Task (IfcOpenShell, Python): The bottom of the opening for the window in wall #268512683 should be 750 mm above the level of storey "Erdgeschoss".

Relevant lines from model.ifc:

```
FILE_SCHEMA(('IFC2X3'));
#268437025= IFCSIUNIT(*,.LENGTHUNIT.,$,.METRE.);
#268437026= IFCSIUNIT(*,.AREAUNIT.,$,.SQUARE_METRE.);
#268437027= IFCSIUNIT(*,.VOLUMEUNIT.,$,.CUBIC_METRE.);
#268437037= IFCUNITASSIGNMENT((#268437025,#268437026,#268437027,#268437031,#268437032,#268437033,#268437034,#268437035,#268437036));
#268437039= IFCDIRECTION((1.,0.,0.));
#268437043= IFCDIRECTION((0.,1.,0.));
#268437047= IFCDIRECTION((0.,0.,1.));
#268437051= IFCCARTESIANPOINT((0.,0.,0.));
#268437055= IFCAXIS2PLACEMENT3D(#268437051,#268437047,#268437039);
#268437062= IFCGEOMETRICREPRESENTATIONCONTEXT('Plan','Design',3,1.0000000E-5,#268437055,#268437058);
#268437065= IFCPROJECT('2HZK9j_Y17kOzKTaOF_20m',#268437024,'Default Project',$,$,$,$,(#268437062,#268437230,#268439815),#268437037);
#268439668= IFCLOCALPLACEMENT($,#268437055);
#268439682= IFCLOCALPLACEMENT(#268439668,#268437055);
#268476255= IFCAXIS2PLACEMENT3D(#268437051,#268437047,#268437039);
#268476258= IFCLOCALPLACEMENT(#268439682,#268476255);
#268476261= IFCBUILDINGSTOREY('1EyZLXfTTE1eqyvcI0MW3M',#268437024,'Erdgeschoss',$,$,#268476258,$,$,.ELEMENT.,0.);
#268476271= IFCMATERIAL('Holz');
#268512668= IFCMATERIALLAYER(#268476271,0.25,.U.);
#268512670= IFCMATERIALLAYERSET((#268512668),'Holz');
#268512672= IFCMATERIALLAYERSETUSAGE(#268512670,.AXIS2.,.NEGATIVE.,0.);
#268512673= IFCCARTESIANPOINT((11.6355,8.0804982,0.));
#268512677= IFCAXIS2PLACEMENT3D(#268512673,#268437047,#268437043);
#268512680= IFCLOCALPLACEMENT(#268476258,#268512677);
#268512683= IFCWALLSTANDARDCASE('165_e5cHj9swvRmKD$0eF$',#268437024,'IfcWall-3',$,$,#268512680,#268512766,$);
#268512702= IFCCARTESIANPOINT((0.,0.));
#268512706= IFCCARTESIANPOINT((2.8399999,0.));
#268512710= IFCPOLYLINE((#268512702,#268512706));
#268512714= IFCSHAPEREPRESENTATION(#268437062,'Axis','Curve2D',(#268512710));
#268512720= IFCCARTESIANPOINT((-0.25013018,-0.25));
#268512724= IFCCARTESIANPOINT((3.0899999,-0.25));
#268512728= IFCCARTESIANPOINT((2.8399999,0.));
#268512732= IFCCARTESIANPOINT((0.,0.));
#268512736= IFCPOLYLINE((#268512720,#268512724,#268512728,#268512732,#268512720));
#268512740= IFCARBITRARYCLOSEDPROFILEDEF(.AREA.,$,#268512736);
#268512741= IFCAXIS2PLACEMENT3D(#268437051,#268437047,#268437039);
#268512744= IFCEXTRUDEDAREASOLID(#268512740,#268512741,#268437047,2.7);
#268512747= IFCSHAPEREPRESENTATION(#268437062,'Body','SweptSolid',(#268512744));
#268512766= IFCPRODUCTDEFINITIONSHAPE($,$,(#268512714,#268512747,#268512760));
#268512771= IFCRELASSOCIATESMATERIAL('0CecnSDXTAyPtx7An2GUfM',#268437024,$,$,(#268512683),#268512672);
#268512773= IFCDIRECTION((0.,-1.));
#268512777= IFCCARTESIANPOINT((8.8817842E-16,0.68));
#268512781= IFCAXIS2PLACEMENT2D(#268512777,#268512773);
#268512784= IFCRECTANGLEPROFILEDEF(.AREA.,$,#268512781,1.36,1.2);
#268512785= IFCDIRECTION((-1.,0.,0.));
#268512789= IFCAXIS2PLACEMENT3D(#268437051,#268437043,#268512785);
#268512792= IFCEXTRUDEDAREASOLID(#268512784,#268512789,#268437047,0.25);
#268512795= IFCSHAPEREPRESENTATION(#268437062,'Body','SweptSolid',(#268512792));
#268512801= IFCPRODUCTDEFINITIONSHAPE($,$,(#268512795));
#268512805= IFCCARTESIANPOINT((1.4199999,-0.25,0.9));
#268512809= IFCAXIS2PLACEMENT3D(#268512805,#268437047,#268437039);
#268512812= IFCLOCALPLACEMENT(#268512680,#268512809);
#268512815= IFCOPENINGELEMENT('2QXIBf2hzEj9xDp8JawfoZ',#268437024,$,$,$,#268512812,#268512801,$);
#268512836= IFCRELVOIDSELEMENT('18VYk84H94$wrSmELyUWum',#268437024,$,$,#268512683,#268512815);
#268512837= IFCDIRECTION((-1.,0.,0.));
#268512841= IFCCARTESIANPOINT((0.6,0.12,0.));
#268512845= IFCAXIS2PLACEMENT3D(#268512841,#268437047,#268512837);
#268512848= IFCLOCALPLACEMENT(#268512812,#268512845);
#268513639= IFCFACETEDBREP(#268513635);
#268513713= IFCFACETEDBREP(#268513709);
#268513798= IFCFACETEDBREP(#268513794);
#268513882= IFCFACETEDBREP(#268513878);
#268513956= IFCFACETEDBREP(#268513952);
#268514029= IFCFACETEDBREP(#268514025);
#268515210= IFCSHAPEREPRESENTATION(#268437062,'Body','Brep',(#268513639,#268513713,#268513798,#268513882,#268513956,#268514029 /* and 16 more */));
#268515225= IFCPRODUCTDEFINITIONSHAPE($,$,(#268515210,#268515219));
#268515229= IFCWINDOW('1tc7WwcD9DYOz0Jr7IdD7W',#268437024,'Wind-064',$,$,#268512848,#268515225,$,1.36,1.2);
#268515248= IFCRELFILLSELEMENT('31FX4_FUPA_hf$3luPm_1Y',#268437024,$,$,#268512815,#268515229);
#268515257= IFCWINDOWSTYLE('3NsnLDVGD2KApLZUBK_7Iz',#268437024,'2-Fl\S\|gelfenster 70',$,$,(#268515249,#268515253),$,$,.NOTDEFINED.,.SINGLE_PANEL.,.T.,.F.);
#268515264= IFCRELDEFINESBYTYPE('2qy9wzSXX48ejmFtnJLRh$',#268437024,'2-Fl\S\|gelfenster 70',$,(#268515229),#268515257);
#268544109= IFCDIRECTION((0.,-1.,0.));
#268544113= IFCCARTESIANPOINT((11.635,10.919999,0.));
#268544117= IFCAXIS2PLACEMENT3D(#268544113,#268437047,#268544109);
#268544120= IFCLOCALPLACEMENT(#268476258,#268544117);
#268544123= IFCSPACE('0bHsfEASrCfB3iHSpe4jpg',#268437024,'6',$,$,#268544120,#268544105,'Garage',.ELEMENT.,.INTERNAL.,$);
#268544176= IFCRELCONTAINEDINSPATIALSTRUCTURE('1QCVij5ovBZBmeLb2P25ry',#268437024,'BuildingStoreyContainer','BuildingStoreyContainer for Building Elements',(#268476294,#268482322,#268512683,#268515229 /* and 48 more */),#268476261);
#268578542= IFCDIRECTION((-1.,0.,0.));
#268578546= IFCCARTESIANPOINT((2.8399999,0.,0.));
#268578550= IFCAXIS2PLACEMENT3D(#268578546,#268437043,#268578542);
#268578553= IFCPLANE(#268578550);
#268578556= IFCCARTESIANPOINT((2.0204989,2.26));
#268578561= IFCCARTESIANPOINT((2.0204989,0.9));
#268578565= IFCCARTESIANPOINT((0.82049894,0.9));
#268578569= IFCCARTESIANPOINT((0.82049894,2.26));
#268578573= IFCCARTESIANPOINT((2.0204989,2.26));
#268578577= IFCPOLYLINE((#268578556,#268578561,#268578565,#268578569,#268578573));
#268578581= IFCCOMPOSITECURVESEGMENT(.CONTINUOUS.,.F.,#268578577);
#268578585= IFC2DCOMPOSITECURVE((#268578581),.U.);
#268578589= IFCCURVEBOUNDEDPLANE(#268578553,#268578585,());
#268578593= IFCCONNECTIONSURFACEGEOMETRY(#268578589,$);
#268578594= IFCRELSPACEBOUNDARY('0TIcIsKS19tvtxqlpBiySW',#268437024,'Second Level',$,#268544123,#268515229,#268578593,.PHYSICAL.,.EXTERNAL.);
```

```python
import numpy as np
import ifcopenshell
import ifcopenshell.api.geometry
import ifcopenshell.geom
import ifcopenshell.util.element
import ifcopenshell.util.placement
import ifcopenshell.util.shape
import ifcopenshell.util.unit

model = ifcopenshell.open("model.ifc")
unit_scale = ifcopenshell.util.unit.calculate_unit_scale(model)

window = model.by_guid("1tc7WwcD9DYOz0Jr7IdD7W")
opening = window.FillsVoids[0].RelatingOpeningElement
storey = ifcopenshell.util.element.get_container(window, ifc_class="IfcBuildingStorey")
level = ifcopenshell.util.placement.get_local_placement(storey.ObjectPlacement)[2, 3]

# The opening's origin need not be at the sill, so measure its lowest point.
shape = ifcopenshell.geom.create_shape(ifcopenshell.geom.settings(), opening)
bottom = ifcopenshell.util.shape.get_shape_bottom_elevation(shape, shape.geometry) / unit_scale
dz = level + 0.75 / unit_scale - bottom

shift = np.array([0.0, 0.0, dz])
# The window is placed relative to its opening, so it follows when the opening moves.
matrix = ifcopenshell.util.placement.get_local_placement(opening.ObjectPlacement)
matrix[:3, 3] += shift
ifcopenshell.api.geometry.edit_object_placement(
    model, product=opening, matrix=matrix, is_si=False, should_transform_children=True
)

# Space boundary surfaces are stored in each space's coordinates; move them too.
for rel in window.ProvidesBoundaries:
    if not rel.ConnectionGeometry:
        continue
    surface = rel.ConnectionGeometry.SurfaceOnRelatingElement.BasisSurface
    space_matrix = ifcopenshell.util.placement.get_local_placement(rel.RelatingSpace.ObjectPlacement)
    point = np.array(surface.Position.Location.Coordinates) + space_matrix[:3, :3].T @ shift
    surface.Position = model.createIfcAxis2Placement3D(
        model.createIfcCartesianPoint(point.tolist()), surface.Position.Axis, surface.Position.RefDirection
    )

print(f"moved by {dz * unit_scale:+.3f} m")

model.write("model_v2.ifc")
```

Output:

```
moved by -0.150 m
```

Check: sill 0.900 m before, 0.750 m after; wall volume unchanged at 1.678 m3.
